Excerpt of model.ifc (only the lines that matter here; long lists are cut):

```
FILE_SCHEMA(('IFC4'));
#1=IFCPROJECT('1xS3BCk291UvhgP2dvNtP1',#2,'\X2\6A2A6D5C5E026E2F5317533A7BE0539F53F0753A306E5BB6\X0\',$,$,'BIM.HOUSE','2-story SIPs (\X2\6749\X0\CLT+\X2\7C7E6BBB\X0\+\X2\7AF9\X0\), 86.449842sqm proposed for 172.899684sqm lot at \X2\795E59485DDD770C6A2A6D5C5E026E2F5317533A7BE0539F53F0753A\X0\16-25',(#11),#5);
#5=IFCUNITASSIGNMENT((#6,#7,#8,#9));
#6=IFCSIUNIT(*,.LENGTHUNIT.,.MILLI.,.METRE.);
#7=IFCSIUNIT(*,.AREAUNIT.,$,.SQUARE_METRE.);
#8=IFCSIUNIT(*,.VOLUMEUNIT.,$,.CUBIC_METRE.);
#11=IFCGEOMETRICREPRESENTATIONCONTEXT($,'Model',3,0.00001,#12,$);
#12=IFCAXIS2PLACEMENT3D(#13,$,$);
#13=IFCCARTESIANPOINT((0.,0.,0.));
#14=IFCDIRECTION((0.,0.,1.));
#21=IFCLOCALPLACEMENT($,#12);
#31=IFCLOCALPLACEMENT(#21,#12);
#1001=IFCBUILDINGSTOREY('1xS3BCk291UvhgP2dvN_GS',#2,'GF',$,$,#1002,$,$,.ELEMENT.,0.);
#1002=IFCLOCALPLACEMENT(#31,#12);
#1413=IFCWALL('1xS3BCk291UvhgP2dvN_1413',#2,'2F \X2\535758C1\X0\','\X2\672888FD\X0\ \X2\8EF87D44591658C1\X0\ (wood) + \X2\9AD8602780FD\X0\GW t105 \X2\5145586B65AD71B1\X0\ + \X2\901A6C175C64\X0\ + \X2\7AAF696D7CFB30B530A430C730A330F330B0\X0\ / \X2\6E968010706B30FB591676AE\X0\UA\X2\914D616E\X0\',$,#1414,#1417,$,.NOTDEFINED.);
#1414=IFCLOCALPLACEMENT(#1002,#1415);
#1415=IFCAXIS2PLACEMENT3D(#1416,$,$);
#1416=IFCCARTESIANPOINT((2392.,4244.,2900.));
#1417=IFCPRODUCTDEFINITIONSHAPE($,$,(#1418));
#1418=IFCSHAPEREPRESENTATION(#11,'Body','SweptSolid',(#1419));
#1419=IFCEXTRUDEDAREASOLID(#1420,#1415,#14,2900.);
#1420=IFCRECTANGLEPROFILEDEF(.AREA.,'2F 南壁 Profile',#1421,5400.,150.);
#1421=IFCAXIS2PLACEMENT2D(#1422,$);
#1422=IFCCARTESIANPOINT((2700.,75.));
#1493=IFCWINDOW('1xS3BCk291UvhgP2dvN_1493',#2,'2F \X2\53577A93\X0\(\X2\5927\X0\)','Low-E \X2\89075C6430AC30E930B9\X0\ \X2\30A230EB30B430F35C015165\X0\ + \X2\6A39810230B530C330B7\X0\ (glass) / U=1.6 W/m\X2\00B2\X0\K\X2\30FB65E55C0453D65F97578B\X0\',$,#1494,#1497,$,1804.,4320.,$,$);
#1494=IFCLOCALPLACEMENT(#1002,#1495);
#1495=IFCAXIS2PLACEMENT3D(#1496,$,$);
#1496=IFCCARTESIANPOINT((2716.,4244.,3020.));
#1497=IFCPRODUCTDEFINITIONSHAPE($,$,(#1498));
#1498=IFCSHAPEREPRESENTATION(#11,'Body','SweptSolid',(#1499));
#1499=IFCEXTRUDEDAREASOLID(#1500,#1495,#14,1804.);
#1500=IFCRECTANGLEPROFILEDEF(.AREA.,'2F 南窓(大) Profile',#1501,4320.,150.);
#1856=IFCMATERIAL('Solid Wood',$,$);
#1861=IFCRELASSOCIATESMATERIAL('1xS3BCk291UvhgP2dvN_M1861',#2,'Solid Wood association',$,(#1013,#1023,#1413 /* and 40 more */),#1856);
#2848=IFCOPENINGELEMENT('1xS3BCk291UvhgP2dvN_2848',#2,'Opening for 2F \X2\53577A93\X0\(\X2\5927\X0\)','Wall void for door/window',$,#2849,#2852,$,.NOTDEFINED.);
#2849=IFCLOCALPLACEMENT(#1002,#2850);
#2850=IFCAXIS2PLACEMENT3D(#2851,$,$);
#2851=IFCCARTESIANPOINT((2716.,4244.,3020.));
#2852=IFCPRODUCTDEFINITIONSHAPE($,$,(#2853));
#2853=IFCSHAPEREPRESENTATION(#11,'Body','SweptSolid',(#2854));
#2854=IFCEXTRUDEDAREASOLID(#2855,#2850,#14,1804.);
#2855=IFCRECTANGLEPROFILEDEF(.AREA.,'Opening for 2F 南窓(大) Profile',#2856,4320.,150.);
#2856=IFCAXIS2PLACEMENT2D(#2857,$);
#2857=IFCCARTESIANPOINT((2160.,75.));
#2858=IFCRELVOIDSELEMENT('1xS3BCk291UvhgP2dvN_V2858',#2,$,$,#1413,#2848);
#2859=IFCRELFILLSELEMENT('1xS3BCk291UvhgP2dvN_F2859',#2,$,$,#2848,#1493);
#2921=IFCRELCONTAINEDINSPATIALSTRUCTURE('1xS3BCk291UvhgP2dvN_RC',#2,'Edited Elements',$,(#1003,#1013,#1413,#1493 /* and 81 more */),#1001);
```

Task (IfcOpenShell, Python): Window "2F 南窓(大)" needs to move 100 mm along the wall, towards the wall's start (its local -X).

```python
import ifcopenshell
import ifcopenshell.api.geometry
import ifcopenshell.util.placement
import ifcopenshell.util.unit

model = ifcopenshell.open("model.ifc")
unit_scale = ifcopenshell.util.unit.calculate_unit_scale(model)

window = model.by_guid("1xS3BCk291UvhgP2dvN_1493")
opening = window.FillsVoids[0].RelatingOpeningElement
wall = opening.VoidsElements[0].RelatingBuildingElement

wall_matrix = ifcopenshell.util.placement.get_local_placement(wall.ObjectPlacement)
shift = wall_matrix[:3, 0] * -0.1 / unit_scale
before = ifcopenshell.util.placement.get_local_placement(window.ObjectPlacement)[:3, 3].copy()

# The window is not placed relative to its opening, so move both.
for product in (opening, window):
    matrix = ifcopenshell.util.placement.get_local_placement(product.ObjectPlacement)
    matrix[:3, 3] += shift
    ifcopenshell.api.geometry.edit_object_placement(model, product=product, matrix=matrix, is_si=False)

after = ifcopenshell.util.placement.get_local_placement(window.ObjectPlacement)[:3, 3]
print("window moved by", (after - before).round(3) + 0.0)

model.write("model_updated.ifc")
```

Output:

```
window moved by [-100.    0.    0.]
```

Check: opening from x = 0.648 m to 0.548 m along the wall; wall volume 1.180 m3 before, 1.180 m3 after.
